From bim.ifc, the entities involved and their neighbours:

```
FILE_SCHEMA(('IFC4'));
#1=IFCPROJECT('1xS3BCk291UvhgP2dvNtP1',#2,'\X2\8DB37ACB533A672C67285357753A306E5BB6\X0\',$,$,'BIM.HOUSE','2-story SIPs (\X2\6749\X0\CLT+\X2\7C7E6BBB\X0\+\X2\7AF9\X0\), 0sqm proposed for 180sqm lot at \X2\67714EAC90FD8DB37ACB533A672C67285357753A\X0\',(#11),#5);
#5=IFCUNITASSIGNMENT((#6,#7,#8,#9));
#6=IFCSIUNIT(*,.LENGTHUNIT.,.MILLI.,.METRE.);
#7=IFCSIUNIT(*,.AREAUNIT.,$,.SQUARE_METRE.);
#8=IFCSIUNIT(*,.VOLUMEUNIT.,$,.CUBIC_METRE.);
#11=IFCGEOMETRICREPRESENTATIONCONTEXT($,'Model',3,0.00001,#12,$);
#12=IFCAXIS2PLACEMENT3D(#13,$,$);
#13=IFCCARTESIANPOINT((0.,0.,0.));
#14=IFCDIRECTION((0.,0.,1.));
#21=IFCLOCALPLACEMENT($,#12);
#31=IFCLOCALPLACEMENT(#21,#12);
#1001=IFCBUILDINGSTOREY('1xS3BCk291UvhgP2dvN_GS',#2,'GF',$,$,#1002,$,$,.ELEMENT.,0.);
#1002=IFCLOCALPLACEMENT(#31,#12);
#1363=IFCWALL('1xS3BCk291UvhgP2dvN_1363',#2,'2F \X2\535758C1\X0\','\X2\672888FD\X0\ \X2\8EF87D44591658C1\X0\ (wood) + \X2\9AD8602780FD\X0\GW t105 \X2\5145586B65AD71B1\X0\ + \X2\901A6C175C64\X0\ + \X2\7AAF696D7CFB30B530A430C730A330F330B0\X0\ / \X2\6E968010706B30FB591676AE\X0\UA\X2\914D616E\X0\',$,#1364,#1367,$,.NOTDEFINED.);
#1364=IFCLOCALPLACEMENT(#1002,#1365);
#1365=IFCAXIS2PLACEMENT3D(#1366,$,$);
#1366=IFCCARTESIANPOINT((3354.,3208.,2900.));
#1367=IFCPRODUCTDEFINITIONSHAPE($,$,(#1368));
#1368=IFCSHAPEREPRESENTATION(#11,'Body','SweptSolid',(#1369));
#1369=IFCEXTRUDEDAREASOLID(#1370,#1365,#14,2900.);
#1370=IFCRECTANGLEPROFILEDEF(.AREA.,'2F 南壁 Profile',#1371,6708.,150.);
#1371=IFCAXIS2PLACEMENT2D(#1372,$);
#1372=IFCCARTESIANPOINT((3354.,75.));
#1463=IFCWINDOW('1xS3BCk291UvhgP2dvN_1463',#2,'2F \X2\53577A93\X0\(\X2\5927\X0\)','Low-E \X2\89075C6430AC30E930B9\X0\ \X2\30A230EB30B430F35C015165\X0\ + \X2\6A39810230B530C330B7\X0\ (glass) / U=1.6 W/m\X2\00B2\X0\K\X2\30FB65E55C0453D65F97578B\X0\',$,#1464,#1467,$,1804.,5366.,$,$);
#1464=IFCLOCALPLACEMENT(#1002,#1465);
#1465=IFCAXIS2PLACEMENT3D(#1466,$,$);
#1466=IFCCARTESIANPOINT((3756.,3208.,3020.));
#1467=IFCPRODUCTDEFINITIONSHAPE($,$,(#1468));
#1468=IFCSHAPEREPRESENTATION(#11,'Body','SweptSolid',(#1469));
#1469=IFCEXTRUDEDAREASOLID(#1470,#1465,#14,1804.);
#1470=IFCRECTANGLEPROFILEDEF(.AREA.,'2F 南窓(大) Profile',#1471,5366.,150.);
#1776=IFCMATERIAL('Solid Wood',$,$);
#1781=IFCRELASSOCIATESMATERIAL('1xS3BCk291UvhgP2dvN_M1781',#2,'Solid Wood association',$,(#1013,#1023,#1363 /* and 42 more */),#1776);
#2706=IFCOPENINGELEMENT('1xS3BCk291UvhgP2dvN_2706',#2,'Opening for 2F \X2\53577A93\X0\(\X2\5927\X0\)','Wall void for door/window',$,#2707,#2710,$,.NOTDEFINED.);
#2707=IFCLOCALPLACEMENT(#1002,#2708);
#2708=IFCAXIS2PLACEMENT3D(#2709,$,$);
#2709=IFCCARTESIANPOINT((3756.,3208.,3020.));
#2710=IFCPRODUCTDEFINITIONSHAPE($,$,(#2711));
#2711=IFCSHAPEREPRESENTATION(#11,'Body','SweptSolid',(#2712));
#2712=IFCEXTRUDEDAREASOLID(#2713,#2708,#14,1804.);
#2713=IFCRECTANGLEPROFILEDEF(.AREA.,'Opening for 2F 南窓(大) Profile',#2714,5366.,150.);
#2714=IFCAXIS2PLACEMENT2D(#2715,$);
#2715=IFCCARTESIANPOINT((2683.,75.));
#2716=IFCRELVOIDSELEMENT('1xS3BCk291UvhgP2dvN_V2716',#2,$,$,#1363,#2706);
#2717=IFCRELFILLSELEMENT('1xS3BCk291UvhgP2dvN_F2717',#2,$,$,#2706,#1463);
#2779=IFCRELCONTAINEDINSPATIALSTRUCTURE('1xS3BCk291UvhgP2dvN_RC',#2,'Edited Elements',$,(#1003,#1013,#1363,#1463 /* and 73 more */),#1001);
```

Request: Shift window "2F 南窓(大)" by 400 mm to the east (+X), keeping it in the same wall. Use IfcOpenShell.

```python
import ifcopenshell
import ifcopenshell.api.geometry
import ifcopenshell.util.placement
import ifcopenshell.util.unit

model = ifcopenshell.open("bim.ifc")
unit_scale = ifcopenshell.util.unit.calculate_unit_scale(model)

window = model.by_guid("1xS3BCk291UvhgP2dvN_1463")
opening = window.FillsVoids[0].RelatingOpeningElement
wall = opening.VoidsElements[0].RelatingBuildingElement

wall_matrix = ifcopenshell.util.placement.get_local_placement(wall.ObjectPlacement)
shift = wall_matrix[:3, 0] * 0.4 / unit_scale
before = ifcopenshell.util.placement.get_local_placement(window.ObjectPlacement)[:3, 3].copy()

# The window is not placed relative to its opening, so move both.
for product in (opening, window):
    matrix = ifcopenshell.util.placement.get_local_placement(product.ObjectPlacement)
    matrix[:3, 3] += shift
    ifcopenshell.api.geometry.edit_object_placement(model, product=product, matrix=matrix, is_si=False)

after = ifcopenshell.util.placement.get_local_placement(window.ObjectPlacement)[:3, 3]
print("window moved by", (after - before).round(3) + 0.0)

model.write("bim_rev.ifc")
```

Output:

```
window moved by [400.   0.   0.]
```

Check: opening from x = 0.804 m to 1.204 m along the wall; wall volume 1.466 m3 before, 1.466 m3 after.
